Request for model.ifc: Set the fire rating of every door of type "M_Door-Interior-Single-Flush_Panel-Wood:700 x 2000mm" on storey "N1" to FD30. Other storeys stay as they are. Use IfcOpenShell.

First a look at what the model holds.

```python
import ifcopenshell
import ifcopenshell.util.element

model = ifcopenshell.open("model.ifc")
print(model.schema)
storey = next(s for s in model.by_type("IfcBuildingStorey") if s.Name == "N1")
doors = [e for e in ifcopenshell.util.element.get_decomposition(storey) if e.is_a("IfcDoor")]
seen = {}
for e in doors:
    element_type = ifcopenshell.util.element.get_type(e)
    key = (element_type.Name if element_type != e and element_type else None, ifcopenshell.util.element.get_pset(e, "Pset_DoorCommon", "FireRating"))
    seen[key] = seen.get(key, 0) + 1
for (name, value), count in sorted(seen.items(), key=str):
    print(count, "x", name, "|", value)
```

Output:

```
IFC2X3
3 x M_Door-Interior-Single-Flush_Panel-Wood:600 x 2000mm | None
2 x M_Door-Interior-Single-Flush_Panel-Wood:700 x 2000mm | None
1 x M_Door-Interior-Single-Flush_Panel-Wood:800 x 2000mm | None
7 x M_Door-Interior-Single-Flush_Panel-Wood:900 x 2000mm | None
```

```python
import ifcopenshell
import ifcopenshell.api.pset
import ifcopenshell.util.element

model = ifcopenshell.open("model.ifc")

storey = next(s for s in model.by_type("IfcBuildingStorey") if s.Name == "N1")
doors = [e for e in ifcopenshell.util.element.get_decomposition(storey) if e.is_a("IfcDoor")]

count = 0
for e in doors:
    element_type = ifcopenshell.util.element.get_type(e)
    if element_type in (None, e) or element_type.Name != "M_Door-Interior-Single-Flush_Panel-Wood:700 x 2000mm":
        continue
    # add_pset returns the element's existing set when there is one.
    pset = ifcopenshell.api.pset.add_pset(model, product=e, name="Pset_DoorCommon")
    ifcopenshell.api.pset.edit_pset(model, pset=pset, properties={"FireRating": "FD30"})
    count += 1

print(count, "doors updated")

model.write("model_v2.ifc")
```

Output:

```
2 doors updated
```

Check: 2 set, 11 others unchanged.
